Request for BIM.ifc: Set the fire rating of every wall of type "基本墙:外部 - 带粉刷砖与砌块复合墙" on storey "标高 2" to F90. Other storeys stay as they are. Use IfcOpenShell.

First a look at what the model holds.

```python
import ifcopenshell
import ifcopenshell.util.element

model = ifcopenshell.open("BIM.ifc")
print(model.schema)
storey = next(s for s in model.by_type("IfcBuildingStorey") if s.Name == "标高 2")
walls = [e for e in ifcopenshell.util.element.get_decomposition(storey) if e.is_a("IfcWall")]
seen = {}
for e in walls:
    element_type = ifcopenshell.util.element.get_type(e)
    key = (element_type.Name if element_type != e and element_type else None, ifcopenshell.util.element.get_pset(e, "Pset_WallCommon", "FireRating"))
    seen[key] = seen.get(key, 0) + 1
for (name, value), count in sorted(seen.items(), key=str):
    print(count, "x", name, "|", value)
```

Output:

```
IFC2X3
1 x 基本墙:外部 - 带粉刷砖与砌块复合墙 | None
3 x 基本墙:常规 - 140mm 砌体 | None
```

```python
import ifcopenshell
import ifcopenshell.api.pset
import ifcopenshell.util.element

model = ifcopenshell.open("BIM.ifc")

storey = next(s for s in model.by_type("IfcBuildingStorey") if s.Name == "标高 2")
walls = [e for e in ifcopenshell.util.element.get_decomposition(storey) if e.is_a("IfcWall")]

count = 0
for e in walls:
    element_type = ifcopenshell.util.element.get_type(e)
    if element_type in (None, e) or element_type.Name != "基本墙:外部 - 带粉刷砖与砌块复合墙":
        continue
    # add_pset returns the element's existing set when there is one.
    pset = ifcopenshell.api.pset.add_pset(model, product=e, name="Pset_WallCommon")
    ifcopenshell.api.pset.edit_pset(model, pset=pset, properties={"FireRating": "F90"})
    count += 1

print(count, "walls updated")

model.write("BIM_rev.ifc")
```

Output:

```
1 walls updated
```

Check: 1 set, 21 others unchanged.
